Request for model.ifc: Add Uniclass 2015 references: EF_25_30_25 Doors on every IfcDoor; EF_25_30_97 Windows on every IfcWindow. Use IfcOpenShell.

First a look at what the model holds.

```python
import ifcopenshell

model = ifcopenshell.open("model.ifc")
print(model.schema)
print("classifications:", [c.Name for c in model.by_type("IfcClassification")])
for ifc_class in ("IfcDoor", "IfcRoof", "IfcStair", "IfcWall", "IfcWindow"):
    print(ifc_class, len(model.by_type(ifc_class)))
```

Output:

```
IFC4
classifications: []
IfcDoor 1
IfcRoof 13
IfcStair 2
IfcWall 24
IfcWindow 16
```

```python
import ifcopenshell
import ifcopenshell.api.classification

model = ifcopenshell.open("model.ifc")

system = ifcopenshell.api.classification.add_classification(model, classification="Uniclass 2015")

codes = {
    "IfcDoor": ("EF_25_30_25", "Doors"),
    "IfcWindow": ("EF_25_30_97", "Windows"),
}
for ifc_class, (code, name) in codes.items():
    products = model.by_type(ifc_class)
    ifcopenshell.api.classification.add_reference(
        model, products=products, classification=system, identification=code, name=name
    )
    print(code, len(products))

model.write("model_edited.ifc")
```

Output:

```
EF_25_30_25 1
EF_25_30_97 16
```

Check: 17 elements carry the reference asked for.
